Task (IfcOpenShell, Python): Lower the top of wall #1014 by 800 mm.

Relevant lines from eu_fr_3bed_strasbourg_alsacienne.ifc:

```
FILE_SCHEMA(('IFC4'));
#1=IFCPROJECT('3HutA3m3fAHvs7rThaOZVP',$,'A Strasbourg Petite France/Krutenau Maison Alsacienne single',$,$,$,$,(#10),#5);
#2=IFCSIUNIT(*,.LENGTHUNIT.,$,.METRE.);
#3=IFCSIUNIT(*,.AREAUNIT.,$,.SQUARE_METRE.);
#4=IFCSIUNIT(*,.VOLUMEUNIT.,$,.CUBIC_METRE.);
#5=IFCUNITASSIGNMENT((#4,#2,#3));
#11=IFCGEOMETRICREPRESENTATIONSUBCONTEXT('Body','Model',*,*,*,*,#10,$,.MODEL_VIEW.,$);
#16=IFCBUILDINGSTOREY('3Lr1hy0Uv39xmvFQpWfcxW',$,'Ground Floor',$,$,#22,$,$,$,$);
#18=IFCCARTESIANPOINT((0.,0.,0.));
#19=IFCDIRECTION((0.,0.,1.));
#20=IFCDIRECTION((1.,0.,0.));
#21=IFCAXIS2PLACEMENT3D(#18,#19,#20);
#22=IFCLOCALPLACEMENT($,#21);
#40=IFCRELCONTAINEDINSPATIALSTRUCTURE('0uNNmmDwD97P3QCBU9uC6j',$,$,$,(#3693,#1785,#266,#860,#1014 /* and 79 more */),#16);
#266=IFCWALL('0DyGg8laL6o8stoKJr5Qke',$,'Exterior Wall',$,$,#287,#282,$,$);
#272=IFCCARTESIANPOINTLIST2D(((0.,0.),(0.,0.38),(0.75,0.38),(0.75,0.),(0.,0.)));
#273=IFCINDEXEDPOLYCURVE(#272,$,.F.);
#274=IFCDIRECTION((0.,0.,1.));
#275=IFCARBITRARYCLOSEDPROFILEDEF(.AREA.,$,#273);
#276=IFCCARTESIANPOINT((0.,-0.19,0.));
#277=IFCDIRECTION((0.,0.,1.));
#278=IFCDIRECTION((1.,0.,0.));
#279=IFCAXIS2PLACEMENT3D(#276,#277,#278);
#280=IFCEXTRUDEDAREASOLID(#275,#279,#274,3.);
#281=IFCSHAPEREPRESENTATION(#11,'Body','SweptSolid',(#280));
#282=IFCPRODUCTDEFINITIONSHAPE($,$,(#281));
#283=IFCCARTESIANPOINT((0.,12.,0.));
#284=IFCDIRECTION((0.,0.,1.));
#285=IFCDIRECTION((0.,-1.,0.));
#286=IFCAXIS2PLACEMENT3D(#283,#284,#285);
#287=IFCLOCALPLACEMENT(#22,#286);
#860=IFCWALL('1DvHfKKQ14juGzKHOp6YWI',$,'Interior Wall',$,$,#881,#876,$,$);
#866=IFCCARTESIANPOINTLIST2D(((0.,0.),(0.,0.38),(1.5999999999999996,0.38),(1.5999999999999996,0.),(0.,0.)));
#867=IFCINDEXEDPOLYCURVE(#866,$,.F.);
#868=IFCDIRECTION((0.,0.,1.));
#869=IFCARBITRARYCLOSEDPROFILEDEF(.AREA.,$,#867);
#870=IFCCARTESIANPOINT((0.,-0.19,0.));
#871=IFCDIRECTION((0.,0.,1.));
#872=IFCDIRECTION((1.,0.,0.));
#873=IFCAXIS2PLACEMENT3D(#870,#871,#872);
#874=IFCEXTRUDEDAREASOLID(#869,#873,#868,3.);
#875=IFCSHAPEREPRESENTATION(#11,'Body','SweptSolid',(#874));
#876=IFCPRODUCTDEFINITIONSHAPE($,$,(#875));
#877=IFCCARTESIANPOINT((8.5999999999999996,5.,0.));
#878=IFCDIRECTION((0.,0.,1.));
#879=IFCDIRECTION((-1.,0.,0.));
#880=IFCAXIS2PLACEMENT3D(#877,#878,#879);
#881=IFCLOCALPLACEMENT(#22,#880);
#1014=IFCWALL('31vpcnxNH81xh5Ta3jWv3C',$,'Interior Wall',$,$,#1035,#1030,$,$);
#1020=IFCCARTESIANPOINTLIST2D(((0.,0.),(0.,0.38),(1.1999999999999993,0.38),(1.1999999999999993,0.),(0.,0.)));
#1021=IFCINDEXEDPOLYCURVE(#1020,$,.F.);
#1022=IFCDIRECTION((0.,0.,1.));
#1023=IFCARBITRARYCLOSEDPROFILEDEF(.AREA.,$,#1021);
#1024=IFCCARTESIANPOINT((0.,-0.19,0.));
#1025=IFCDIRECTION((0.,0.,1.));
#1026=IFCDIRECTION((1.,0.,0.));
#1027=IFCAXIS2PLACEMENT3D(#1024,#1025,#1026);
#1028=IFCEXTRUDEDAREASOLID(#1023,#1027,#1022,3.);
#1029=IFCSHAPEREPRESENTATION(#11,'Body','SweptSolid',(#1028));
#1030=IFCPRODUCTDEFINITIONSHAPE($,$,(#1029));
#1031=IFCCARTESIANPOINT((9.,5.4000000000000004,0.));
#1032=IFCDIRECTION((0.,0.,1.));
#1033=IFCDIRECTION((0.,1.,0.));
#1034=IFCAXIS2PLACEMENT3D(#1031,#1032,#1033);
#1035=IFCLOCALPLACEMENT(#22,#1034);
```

```python
import ifcopenshell
import ifcopenshell.geom
import ifcopenshell.util.representation
import ifcopenshell.util.shape
import ifcopenshell.util.unit

model = ifcopenshell.open("eu_fr_3bed_strasbourg_alsacienne.ifc")
unit_scale = ifcopenshell.util.unit.calculate_unit_scale(model)
settings = ifcopenshell.geom.settings()


def volume(element):
    """Net volume in cubic metres, openings subtracted."""
    shape = ifcopenshell.geom.create_shape(settings, element)
    return ifcopenshell.util.shape.get_volume(shape.geometry)


wall = model.by_guid("31vpcnxNH81xh5Ta3jWv3C")
before = volume(wall)

body = ifcopenshell.util.representation.get_representation(wall, "Model", "Body")
solid = body.Items[0]
old_height = solid.Depth
solid.Depth -= 0.8 / unit_scale
after = volume(wall)

print(f"height {old_height:g} -> {solid.Depth:g}, volume {before:.3f} -> {after:.3f} m3")

model.write("eu_fr_3bed_strasbourg_alsacienne_updated.ifc")
```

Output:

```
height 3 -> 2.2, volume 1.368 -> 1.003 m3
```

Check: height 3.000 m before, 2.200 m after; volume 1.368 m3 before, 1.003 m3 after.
